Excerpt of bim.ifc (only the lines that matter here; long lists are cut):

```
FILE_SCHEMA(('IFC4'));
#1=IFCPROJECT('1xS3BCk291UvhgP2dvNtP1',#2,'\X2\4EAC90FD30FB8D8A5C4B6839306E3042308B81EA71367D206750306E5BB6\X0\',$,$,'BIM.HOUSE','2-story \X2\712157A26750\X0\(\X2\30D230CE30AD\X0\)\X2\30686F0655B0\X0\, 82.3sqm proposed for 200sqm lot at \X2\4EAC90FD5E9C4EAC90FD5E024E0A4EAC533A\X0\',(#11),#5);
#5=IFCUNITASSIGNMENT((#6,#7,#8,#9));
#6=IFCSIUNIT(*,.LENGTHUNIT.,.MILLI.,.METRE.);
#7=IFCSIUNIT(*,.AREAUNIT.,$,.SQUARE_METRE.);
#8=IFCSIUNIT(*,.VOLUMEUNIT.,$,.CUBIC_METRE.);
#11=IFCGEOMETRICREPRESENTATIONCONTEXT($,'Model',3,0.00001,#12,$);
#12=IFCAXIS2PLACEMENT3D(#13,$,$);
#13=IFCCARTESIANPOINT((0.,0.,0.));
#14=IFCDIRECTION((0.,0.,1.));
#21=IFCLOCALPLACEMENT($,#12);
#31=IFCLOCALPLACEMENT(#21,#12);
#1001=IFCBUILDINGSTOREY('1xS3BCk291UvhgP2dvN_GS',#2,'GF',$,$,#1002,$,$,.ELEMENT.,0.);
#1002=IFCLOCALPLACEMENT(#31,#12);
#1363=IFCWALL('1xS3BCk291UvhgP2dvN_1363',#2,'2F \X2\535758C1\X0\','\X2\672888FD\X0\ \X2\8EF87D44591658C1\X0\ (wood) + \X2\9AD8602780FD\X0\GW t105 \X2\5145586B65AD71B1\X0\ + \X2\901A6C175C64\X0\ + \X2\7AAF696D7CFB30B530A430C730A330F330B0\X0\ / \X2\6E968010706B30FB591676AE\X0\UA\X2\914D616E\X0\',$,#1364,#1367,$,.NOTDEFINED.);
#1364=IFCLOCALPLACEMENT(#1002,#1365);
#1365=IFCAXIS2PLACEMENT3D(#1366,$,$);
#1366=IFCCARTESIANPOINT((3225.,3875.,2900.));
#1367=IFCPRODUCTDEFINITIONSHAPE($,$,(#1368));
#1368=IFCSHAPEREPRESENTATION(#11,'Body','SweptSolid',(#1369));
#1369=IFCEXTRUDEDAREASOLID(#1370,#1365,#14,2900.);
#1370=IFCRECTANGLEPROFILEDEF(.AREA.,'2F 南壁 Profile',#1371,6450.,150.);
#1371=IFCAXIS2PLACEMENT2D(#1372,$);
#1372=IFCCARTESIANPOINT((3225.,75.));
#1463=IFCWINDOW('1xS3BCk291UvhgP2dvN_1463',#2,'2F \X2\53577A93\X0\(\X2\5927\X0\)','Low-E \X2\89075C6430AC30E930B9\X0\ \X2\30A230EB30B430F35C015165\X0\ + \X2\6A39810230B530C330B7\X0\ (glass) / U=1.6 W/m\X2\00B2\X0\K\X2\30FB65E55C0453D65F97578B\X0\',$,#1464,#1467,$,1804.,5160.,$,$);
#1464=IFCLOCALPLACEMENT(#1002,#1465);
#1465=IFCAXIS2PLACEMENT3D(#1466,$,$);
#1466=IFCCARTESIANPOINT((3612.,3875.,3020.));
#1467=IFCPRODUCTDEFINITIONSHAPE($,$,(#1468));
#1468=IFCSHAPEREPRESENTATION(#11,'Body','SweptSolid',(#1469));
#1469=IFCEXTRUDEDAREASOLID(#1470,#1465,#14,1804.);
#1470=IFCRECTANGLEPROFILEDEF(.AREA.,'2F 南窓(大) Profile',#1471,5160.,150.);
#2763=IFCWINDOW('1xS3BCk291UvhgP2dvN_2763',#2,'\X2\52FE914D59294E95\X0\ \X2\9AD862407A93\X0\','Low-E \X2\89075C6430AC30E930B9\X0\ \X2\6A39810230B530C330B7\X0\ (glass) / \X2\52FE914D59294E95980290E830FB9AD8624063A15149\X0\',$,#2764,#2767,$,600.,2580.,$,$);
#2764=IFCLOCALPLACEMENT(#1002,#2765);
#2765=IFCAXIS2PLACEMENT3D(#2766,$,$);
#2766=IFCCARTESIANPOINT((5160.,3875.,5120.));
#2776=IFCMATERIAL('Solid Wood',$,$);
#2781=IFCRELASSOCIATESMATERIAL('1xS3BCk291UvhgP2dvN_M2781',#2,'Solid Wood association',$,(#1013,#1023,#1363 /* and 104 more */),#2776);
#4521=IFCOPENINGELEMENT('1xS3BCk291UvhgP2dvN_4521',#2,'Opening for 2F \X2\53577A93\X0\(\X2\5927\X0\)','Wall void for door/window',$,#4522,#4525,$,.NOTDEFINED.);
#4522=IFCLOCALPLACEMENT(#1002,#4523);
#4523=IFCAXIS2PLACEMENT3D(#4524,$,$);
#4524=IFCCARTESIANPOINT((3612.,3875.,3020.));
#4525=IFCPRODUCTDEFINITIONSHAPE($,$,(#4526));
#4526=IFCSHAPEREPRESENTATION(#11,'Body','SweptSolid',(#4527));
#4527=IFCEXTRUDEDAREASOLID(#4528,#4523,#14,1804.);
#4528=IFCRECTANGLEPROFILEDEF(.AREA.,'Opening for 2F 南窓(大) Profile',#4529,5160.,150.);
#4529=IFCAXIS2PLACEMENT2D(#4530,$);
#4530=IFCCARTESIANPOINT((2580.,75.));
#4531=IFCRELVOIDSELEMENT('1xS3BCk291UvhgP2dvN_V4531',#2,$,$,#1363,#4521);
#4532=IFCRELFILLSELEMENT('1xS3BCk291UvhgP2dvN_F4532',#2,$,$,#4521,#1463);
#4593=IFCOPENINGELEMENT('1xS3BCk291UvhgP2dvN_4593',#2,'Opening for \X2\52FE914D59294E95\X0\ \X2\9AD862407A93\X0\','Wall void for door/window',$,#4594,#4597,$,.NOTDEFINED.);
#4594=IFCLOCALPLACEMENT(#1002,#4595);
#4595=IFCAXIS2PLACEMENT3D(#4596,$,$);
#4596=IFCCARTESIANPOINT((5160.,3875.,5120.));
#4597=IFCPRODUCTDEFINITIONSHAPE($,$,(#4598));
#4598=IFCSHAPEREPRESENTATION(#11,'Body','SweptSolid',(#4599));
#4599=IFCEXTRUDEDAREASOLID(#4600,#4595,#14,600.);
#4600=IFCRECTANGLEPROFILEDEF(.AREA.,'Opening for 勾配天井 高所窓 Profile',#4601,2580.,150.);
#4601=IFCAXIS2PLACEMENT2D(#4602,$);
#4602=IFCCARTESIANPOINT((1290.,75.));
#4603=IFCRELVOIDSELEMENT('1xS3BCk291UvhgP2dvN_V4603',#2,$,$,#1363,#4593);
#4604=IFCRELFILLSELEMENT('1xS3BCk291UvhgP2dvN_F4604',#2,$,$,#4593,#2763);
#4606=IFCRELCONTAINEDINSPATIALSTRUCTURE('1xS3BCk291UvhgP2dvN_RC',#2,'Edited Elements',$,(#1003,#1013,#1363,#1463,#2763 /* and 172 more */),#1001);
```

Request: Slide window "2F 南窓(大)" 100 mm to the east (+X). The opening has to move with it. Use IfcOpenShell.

```python
import ifcopenshell
import ifcopenshell.api.geometry
import ifcopenshell.util.placement
import ifcopenshell.util.unit

model = ifcopenshell.open("bim.ifc")
unit_scale = ifcopenshell.util.unit.calculate_unit_scale(model)

window = model.by_id(1463)
opening = window.FillsVoids[0].RelatingOpeningElement
wall = opening.VoidsElements[0].RelatingBuildingElement

wall_matrix = ifcopenshell.util.placement.get_local_placement(wall.ObjectPlacement)
shift = wall_matrix[:3, 0] * 0.1 / unit_scale
before = ifcopenshell.util.placement.get_local_placement(window.ObjectPlacement)[:3, 3].copy()

# The window is not placed relative to its opening, so move both.
for product in (opening, window):
    matrix = ifcopenshell.util.placement.get_local_placement(product.ObjectPlacement)
    matrix[:3, 3] += shift
    ifcopenshell.api.geometry.edit_object_placement(model, product=product, matrix=matrix, is_si=False)

after = ifcopenshell.util.placement.get_local_placement(window.ObjectPlacement)[:3, 3]
print("window moved by", (after - before).round(3) + 0.0)

model.write("bim_edited.ifc")
```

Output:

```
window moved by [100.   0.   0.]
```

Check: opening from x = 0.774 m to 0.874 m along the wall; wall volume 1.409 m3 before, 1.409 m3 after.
